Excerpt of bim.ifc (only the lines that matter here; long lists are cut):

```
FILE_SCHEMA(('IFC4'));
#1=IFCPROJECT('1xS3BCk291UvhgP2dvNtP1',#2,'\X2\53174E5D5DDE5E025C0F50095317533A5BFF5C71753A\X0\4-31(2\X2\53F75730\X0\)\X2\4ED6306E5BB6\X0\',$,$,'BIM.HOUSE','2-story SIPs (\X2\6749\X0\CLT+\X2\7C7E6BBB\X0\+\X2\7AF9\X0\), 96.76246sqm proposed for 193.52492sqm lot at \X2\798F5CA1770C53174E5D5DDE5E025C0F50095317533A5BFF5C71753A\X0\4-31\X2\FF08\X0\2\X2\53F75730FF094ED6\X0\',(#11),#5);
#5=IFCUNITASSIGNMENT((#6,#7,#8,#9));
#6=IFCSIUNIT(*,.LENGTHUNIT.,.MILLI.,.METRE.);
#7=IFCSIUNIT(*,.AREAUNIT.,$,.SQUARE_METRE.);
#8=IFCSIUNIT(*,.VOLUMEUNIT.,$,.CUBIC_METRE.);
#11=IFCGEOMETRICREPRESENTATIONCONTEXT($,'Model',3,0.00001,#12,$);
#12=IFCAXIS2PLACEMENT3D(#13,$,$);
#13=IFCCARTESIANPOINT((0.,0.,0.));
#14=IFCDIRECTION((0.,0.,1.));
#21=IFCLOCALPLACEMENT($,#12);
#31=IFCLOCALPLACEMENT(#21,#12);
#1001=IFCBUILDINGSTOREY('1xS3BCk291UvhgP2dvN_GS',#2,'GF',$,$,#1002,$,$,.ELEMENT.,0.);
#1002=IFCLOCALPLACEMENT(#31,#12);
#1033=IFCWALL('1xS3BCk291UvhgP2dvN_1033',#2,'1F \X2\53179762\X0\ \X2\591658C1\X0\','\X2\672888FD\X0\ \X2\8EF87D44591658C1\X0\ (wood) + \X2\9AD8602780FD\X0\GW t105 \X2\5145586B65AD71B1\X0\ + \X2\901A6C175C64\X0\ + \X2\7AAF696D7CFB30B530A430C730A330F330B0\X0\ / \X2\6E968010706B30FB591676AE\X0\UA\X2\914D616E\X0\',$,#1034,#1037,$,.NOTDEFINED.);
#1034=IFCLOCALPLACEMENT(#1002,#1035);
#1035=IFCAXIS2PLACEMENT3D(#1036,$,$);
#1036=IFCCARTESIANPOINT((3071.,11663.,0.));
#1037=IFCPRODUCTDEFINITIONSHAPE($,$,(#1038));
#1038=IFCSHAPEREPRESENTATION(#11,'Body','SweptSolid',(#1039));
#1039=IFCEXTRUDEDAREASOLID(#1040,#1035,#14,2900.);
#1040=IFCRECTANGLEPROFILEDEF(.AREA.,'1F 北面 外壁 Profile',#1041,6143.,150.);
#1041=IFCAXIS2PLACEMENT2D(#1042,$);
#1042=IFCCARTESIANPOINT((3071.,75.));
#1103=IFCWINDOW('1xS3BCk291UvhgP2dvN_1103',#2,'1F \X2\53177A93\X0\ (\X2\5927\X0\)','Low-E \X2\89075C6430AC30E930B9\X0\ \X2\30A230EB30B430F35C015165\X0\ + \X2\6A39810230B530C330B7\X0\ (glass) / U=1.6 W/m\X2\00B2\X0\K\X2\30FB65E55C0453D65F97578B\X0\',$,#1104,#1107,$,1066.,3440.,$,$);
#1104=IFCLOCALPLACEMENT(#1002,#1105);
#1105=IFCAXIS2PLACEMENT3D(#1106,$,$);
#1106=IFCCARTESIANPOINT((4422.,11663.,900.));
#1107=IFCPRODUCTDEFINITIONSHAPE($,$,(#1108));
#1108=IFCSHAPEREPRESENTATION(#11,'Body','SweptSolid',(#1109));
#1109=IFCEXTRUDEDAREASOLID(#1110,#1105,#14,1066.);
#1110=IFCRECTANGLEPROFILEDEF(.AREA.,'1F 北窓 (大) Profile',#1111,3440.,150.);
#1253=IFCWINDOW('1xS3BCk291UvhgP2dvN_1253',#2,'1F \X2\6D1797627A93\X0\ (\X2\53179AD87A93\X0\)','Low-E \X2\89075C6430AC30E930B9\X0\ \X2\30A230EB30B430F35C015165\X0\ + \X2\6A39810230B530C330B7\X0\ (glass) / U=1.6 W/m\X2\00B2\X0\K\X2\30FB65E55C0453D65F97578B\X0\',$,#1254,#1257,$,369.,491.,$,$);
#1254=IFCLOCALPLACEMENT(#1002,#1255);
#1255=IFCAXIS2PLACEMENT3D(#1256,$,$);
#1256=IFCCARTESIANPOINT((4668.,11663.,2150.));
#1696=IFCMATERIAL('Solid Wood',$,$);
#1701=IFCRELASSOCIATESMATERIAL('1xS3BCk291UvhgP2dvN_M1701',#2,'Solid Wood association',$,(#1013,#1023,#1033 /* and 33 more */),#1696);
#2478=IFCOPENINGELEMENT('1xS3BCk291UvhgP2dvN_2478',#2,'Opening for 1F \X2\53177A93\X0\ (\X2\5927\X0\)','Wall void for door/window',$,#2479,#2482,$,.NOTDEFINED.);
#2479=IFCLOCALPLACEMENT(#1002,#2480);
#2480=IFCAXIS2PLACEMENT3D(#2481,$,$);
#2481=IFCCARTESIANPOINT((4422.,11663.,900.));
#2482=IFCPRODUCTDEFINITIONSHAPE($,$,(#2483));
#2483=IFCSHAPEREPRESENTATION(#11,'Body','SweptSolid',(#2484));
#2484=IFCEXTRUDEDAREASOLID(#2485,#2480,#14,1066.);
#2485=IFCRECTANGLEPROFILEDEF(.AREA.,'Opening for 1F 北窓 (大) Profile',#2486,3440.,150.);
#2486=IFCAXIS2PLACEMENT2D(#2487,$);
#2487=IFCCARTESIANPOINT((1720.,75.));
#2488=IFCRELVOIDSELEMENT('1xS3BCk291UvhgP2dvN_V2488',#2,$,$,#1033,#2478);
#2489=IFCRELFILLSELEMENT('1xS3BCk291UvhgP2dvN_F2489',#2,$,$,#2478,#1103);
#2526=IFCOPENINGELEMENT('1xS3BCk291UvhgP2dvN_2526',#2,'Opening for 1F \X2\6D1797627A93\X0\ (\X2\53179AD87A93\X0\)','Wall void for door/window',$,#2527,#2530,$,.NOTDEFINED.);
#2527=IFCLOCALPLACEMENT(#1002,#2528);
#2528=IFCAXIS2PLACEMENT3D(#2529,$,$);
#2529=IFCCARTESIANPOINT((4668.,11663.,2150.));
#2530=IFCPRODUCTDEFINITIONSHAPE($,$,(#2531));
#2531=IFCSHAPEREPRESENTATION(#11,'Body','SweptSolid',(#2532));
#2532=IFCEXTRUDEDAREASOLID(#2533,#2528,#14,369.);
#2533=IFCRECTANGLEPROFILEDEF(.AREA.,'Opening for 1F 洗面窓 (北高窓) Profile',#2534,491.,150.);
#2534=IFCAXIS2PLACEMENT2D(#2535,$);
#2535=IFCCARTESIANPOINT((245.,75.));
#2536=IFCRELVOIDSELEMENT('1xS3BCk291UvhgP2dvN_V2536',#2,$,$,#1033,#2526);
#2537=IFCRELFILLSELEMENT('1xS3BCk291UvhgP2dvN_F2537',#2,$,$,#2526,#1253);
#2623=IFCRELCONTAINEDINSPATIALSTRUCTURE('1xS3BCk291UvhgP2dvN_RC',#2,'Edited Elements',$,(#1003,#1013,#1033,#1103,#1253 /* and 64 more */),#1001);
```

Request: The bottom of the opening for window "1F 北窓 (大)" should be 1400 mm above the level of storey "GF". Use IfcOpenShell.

```python
import numpy as np
import ifcopenshell
import ifcopenshell.api.geometry
import ifcopenshell.geom
import ifcopenshell.util.element
import ifcopenshell.util.placement
import ifcopenshell.util.shape
import ifcopenshell.util.unit

model = ifcopenshell.open("bim.ifc")
unit_scale = ifcopenshell.util.unit.calculate_unit_scale(model)

window = model.by_guid("1xS3BCk291UvhgP2dvN_1103")
opening = window.FillsVoids[0].RelatingOpeningElement
storey = ifcopenshell.util.element.get_container(window, ifc_class="IfcBuildingStorey")
level = ifcopenshell.util.placement.get_local_placement(storey.ObjectPlacement)[2, 3]

# The opening's origin need not be at the sill, so measure its lowest point.
shape = ifcopenshell.geom.create_shape(ifcopenshell.geom.settings(), opening)
bottom = ifcopenshell.util.shape.get_shape_bottom_elevation(shape, shape.geometry) / unit_scale
dz = level + 1400.0 - bottom

shift = np.array([0.0, 0.0, dz])
# The window is not placed relative to its opening, so move both.
for product in (opening, window):
    matrix = ifcopenshell.util.placement.get_local_placement(product.ObjectPlacement)
    matrix[:3, 3] += shift
    ifcopenshell.api.geometry.edit_object_placement(model, product=product, matrix=matrix, is_si=False)

print(f"moved by {dz * unit_scale:+.3f} m")

model.write("bim_updated.ifc")
```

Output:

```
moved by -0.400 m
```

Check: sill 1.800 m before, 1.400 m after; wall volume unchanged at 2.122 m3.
